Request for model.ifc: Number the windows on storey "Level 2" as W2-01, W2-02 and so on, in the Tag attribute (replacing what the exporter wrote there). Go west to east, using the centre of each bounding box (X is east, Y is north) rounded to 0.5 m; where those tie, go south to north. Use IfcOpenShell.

First a look at what the model holds.

```python
import ifcopenshell
import ifcopenshell.util.element
import ifcopenshell.util.placement

model = ifcopenshell.open("model.ifc")
print(model.schema)
storey = next(s for s in model.by_type("IfcBuildingStorey") if s.Name == "Level 2")
windows = [e for e in ifcopenshell.util.element.get_decomposition(storey) if e.is_a("IfcWindow")]
for e in sorted(windows, key=lambda e: e.id()):
    origin = ifcopenshell.util.placement.get_local_placement(e.ObjectPlacement)[:3, 3]
    print(e.id(), e.Tag, e.Name, origin.round(2) + 0.0, sep=" | ")
```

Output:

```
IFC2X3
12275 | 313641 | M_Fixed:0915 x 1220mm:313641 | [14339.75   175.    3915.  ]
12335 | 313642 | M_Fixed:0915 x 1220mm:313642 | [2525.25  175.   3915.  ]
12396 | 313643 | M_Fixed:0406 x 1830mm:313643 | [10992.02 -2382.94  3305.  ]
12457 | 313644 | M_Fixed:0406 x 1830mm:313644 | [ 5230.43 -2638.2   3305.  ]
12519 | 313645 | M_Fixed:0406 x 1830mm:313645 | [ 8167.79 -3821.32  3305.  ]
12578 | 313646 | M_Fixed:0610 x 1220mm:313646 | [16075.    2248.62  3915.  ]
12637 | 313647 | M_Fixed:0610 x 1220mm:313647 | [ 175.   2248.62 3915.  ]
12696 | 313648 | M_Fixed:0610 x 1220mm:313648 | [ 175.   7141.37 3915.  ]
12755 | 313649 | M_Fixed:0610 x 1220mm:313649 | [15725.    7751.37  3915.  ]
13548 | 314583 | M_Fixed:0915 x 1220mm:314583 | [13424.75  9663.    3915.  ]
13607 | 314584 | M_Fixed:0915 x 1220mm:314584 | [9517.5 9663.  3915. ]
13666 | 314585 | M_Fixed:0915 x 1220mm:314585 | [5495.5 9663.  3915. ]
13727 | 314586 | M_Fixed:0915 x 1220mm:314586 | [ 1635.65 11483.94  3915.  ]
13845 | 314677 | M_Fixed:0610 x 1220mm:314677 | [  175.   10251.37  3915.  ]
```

```python
import ifcopenshell
import ifcopenshell.geom
import ifcopenshell.util.element
import ifcopenshell.util.shape

model = ifcopenshell.open("model.ifc")
settings = ifcopenshell.geom.settings()
settings.set("use-world-coords", True)


def centre(element):
    shape = ifcopenshell.geom.create_shape(settings, element)
    return ifcopenshell.util.shape.get_bbox_centroid(shape.geometry)


storey = next(s for s in model.by_type("IfcBuildingStorey") if s.Name == "Level 2")
windows = [e for e in ifcopenshell.util.element.get_decomposition(storey) if e.is_a("IfcWindow")]

# Insertion points can sit at a corner or the storey origin, so sort by the geometry (in metres).
centres = {e: centre(e) for e in windows}
windows.sort(key=lambda e: (round(centres[e][0] / 0.5), centres[e][1]))

for i, e in enumerate(windows, start=1):
    number = f"W2-{i:02d}"
    e.Tag = number
    print(e.id(), number)

model.write("model_updated.ifc")
```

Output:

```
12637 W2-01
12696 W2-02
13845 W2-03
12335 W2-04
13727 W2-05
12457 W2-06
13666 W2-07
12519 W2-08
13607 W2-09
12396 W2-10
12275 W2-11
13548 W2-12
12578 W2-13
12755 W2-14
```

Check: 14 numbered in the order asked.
